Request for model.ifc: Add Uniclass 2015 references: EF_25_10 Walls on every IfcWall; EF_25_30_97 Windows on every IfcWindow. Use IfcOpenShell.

First a look at what the model holds.

```python
import ifcopenshell

model = ifcopenshell.open("model.ifc")
print(model.schema)
print("classifications:", [c.Name for c in model.by_type("IfcClassification")])
for ifc_class in ("IfcDoor", "IfcRoof", "IfcStair", "IfcWall", "IfcWindow"):
    print(ifc_class, len(model.by_type(ifc_class)))
```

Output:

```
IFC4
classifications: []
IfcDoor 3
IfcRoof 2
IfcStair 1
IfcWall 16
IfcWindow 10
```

```python
import ifcopenshell
import ifcopenshell.api.classification

model = ifcopenshell.open("model.ifc")

system = ifcopenshell.api.classification.add_classification(model, classification="Uniclass 2015")

codes = {
    "IfcWall": ("EF_25_10", "Walls"),
    "IfcWindow": ("EF_25_30_97", "Windows"),
}
for ifc_class, (code, name) in codes.items():
    products = model.by_type(ifc_class)
    ifcopenshell.api.classification.add_reference(
        model, products=products, classification=system, identification=code, name=name
    )
    print(code, len(products))

model.write("model-out.ifc")
```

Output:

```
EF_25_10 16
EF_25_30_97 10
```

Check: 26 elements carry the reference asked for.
